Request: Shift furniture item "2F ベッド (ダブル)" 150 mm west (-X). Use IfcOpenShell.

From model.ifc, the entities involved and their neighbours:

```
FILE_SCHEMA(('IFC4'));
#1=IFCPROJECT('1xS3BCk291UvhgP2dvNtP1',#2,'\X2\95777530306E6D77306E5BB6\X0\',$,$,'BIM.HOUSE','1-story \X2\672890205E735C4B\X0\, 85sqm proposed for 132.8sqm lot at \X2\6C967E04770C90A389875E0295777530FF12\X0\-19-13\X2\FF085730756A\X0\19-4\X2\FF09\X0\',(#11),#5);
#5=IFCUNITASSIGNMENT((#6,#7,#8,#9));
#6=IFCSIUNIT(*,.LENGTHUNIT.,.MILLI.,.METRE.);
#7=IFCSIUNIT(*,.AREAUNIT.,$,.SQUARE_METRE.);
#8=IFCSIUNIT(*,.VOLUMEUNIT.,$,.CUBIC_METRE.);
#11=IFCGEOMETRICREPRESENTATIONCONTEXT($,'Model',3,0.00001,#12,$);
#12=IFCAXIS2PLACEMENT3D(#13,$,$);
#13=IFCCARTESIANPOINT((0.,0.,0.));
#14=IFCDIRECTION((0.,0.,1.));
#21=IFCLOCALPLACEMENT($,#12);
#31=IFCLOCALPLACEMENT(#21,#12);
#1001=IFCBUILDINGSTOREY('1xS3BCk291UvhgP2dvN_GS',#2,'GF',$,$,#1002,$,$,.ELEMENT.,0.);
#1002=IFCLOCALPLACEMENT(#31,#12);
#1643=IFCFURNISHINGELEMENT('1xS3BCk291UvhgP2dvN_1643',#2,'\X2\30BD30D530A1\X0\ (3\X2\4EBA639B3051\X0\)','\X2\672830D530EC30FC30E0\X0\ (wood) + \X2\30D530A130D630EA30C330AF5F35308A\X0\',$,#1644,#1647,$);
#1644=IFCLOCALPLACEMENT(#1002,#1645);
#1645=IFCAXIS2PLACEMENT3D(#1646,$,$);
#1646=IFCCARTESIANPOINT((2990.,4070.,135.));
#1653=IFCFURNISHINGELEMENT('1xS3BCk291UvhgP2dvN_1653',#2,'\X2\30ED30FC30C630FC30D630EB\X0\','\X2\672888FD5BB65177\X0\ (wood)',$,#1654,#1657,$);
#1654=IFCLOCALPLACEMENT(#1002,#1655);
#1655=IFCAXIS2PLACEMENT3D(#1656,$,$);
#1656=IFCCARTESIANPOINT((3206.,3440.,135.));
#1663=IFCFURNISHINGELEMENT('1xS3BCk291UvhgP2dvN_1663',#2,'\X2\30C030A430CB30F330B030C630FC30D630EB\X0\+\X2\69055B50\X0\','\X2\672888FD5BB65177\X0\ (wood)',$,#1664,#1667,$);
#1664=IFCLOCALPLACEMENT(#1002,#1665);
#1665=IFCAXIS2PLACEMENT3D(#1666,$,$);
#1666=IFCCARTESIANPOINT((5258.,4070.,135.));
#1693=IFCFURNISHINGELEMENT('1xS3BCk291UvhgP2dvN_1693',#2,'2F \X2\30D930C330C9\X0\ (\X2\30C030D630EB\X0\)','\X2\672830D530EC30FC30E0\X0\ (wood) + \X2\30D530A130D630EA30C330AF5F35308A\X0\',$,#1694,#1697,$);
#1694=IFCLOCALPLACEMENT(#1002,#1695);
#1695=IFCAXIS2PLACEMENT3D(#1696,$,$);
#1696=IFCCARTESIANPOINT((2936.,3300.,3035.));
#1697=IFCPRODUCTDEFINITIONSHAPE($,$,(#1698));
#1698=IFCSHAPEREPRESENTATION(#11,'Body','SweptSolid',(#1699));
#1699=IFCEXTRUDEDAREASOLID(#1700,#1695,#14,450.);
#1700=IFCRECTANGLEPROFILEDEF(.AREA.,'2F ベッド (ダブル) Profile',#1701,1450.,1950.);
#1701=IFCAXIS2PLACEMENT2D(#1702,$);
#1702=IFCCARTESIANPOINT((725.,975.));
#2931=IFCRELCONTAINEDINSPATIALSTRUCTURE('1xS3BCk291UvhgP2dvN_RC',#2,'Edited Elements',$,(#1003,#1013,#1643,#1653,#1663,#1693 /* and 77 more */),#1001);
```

```python
import ifcopenshell
import ifcopenshell.api.geometry
import ifcopenshell.util.placement
import ifcopenshell.util.unit

model = ifcopenshell.open("model.ifc")
unit_scale = ifcopenshell.util.unit.calculate_unit_scale(model)

item = model.by_guid("1xS3BCk291UvhgP2dvN_1693")
matrix = ifcopenshell.util.placement.get_local_placement(item.ObjectPlacement)
matrix[0, 3] -= 0.15 / unit_scale
ifcopenshell.api.geometry.edit_object_placement(model, product=item, matrix=matrix, is_si=False)

print(ifcopenshell.util.placement.get_local_placement(item.ObjectPlacement).round(3) + 0.0)

model.write("model_updated.ifc")
```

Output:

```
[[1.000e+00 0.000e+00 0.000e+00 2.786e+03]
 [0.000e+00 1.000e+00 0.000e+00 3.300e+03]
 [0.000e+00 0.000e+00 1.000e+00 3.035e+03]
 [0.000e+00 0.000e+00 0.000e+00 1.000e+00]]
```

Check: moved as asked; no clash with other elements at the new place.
